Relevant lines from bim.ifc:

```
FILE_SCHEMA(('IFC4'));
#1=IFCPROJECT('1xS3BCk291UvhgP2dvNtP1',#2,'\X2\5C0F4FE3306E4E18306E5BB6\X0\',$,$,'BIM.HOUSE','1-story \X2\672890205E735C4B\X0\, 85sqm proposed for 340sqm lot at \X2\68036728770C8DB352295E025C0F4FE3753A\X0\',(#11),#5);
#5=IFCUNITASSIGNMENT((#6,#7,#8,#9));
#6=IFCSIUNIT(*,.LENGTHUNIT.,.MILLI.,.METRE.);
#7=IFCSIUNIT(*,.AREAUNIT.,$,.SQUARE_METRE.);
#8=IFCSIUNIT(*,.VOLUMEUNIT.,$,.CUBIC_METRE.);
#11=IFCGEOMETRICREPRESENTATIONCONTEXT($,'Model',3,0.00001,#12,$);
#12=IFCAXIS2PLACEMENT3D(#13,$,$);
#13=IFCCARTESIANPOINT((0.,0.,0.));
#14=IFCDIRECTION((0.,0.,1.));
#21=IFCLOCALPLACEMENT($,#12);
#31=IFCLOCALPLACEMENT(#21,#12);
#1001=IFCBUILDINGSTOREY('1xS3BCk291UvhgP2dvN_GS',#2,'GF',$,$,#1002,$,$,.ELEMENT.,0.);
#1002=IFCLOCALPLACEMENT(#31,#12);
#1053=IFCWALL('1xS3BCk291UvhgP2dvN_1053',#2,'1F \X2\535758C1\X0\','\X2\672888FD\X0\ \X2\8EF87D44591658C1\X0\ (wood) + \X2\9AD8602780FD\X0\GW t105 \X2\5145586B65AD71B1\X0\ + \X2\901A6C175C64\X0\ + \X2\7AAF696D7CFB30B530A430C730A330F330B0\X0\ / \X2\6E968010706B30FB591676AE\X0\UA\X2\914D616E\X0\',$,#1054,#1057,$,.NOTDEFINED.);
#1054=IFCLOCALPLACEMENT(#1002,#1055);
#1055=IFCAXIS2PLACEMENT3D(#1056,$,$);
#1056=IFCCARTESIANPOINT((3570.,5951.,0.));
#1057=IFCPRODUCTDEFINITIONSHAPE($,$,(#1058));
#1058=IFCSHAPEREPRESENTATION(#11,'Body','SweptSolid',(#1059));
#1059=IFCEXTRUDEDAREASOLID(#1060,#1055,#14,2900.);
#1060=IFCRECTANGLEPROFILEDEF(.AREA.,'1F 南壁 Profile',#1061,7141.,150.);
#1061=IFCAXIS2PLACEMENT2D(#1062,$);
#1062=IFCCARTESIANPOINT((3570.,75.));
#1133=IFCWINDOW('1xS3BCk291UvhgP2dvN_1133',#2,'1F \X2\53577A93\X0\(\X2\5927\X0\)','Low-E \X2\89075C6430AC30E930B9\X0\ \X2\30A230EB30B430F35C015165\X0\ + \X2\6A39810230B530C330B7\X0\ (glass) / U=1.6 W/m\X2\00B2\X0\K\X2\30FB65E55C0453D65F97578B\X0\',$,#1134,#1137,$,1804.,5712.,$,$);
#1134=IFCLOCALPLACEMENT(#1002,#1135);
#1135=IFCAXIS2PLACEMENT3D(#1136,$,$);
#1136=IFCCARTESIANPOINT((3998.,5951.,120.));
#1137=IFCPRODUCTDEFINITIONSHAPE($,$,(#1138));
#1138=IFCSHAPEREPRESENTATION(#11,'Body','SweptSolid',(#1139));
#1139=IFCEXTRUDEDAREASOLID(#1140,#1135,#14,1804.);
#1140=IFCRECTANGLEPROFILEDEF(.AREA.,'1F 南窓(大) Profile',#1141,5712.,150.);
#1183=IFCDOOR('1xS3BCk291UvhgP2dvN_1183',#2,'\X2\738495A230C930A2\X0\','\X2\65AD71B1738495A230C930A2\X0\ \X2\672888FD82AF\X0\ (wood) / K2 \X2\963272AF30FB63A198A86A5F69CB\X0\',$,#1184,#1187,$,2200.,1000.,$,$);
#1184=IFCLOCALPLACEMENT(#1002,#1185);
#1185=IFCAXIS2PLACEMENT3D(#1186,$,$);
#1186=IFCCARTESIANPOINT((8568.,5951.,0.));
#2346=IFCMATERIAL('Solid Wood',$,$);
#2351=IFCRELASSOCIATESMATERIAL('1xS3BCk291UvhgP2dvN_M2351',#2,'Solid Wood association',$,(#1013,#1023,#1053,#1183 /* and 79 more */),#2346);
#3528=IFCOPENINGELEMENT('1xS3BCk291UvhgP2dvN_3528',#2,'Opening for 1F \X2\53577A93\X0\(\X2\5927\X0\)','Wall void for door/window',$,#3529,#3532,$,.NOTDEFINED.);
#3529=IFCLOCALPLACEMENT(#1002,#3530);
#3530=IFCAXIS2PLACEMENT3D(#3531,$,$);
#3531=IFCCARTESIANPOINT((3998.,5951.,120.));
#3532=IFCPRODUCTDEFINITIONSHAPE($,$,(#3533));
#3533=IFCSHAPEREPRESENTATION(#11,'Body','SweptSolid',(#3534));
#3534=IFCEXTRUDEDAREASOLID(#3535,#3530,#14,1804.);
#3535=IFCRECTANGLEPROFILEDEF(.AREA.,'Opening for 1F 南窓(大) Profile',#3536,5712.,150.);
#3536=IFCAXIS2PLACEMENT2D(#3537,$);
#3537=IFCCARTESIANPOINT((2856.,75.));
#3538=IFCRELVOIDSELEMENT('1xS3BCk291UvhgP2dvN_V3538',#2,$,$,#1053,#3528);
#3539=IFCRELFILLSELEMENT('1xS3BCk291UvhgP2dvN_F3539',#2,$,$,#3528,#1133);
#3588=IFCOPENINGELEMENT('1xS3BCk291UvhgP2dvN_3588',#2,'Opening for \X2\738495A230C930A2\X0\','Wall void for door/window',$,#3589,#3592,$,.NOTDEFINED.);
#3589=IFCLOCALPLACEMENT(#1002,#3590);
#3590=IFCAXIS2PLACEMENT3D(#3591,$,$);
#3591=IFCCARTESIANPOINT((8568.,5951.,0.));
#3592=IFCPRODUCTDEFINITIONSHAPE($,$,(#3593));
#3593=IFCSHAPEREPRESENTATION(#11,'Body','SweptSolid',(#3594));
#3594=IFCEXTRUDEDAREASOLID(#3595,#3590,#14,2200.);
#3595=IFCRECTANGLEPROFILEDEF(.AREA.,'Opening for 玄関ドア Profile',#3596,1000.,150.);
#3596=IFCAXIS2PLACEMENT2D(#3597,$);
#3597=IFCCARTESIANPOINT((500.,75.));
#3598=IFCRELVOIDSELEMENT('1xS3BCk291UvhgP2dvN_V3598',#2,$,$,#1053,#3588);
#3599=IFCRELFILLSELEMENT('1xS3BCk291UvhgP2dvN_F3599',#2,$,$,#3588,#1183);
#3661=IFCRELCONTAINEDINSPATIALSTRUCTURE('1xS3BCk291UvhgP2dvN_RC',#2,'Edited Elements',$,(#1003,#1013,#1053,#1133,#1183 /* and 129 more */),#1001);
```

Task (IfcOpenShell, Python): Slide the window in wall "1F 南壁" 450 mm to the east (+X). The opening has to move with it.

```python
import ifcopenshell
import ifcopenshell.api.geometry
import ifcopenshell.util.placement

model = ifcopenshell.open("bim.ifc")

window = model.by_id(1133)
opening = window.FillsVoids[0].RelatingOpeningElement
wall = opening.VoidsElements[0].RelatingBuildingElement

wall_matrix = ifcopenshell.util.placement.get_local_placement(wall.ObjectPlacement)
shift = wall_matrix[:3, 0] * 450.0
before = ifcopenshell.util.placement.get_local_placement(window.ObjectPlacement)[:3, 3].copy()

# The window is not placed relative to its opening, so move both.
for product in (opening, window):
    matrix = ifcopenshell.util.placement.get_local_placement(product.ObjectPlacement)
    matrix[:3, 3] += shift
    ifcopenshell.api.geometry.edit_object_placement(model, product=product, matrix=matrix, is_si=False)

after = ifcopenshell.util.placement.get_local_placement(window.ObjectPlacement)[:3, 3]
print("window moved by", (after - before).round(3) + 0.0)

model.write("bim_v2.ifc")
```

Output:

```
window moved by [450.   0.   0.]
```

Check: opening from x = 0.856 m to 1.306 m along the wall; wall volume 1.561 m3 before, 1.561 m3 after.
